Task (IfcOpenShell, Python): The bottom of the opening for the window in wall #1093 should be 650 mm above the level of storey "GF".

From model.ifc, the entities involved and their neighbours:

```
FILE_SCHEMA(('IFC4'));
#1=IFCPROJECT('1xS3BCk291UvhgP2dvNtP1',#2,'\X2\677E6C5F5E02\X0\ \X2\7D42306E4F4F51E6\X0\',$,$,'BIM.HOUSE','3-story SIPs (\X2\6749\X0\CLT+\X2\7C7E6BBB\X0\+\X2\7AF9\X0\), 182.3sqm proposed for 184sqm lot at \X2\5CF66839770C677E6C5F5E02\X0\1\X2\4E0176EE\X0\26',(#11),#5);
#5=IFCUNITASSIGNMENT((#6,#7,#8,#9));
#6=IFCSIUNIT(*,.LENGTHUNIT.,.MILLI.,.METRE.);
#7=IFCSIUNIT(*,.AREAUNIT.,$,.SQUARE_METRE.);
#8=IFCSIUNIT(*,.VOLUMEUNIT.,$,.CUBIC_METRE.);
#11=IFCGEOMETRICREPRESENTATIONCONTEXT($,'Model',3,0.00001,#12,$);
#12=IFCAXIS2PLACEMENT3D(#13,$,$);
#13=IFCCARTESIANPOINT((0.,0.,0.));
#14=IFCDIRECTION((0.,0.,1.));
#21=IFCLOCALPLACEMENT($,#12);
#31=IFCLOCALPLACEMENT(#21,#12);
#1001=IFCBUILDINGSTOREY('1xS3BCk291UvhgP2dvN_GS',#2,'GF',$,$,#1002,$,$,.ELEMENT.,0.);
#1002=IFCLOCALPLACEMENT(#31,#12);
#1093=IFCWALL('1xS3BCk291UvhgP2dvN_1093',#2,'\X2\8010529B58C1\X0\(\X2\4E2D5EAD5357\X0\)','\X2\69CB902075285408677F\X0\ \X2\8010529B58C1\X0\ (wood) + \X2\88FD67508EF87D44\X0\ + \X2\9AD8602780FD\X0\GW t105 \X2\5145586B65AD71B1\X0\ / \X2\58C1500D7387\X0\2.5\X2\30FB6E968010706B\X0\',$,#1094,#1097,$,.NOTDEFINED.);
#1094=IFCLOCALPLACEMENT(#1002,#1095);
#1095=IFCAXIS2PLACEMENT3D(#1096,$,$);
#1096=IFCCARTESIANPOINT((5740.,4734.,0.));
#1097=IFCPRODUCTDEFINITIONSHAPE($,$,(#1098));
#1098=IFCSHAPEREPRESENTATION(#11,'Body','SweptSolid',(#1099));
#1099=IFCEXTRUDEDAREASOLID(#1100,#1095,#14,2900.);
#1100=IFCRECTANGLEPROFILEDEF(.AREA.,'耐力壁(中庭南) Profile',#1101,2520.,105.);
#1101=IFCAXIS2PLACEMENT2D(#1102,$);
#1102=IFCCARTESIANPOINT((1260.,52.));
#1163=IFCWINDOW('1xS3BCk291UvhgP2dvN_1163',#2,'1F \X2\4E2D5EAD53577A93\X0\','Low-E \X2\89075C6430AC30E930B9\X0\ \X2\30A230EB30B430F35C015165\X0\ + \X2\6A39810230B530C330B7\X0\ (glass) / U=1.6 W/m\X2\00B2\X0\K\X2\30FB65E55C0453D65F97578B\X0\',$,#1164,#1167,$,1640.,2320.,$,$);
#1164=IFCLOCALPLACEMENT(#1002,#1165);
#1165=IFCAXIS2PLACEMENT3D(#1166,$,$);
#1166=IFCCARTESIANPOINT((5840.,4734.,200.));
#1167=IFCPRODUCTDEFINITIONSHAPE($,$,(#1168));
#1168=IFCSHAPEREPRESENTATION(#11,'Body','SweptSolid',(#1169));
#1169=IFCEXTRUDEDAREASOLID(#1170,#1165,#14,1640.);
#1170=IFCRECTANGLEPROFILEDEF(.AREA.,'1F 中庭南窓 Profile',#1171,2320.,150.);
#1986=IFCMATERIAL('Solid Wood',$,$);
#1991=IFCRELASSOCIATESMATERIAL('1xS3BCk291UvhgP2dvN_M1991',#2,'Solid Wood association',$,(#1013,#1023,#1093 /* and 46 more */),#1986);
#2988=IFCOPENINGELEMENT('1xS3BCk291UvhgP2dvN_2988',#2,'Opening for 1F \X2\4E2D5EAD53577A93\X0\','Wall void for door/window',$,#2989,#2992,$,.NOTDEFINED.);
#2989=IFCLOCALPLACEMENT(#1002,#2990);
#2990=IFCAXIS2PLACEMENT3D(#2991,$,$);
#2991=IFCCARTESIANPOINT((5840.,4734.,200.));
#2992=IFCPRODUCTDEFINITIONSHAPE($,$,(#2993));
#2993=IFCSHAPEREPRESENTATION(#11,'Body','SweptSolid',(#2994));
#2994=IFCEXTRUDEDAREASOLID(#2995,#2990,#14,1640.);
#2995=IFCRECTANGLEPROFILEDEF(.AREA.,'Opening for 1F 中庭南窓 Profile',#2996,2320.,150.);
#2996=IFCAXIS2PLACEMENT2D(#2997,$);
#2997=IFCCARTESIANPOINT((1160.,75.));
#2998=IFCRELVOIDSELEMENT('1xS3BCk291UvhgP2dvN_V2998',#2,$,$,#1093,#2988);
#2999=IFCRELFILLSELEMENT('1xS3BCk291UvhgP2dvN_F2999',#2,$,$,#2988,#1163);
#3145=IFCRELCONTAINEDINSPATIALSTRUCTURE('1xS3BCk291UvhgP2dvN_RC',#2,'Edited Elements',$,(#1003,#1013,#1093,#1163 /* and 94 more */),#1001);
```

```python
import numpy as np
import ifcopenshell
import ifcopenshell.api.geometry
import ifcopenshell.geom
import ifcopenshell.util.element
import ifcopenshell.util.placement
import ifcopenshell.util.shape
import ifcopenshell.util.unit

model = ifcopenshell.open("model.ifc")
unit_scale = ifcopenshell.util.unit.calculate_unit_scale(model)

window = model.by_id(1163)
opening = window.FillsVoids[0].RelatingOpeningElement
storey = ifcopenshell.util.element.get_container(window, ifc_class="IfcBuildingStorey")
level = ifcopenshell.util.placement.get_local_placement(storey.ObjectPlacement)[2, 3]

# The opening's origin need not be at the sill, so measure its lowest point.
shape = ifcopenshell.geom.create_shape(ifcopenshell.geom.settings(), opening)
bottom = ifcopenshell.util.shape.get_shape_bottom_elevation(shape, shape.geometry) / unit_scale
dz = level + 0.65 / unit_scale - bottom

shift = np.array([0.0, 0.0, dz])
# The window is not placed relative to its opening, so move both.
for product in (opening, window):
    matrix = ifcopenshell.util.placement.get_local_placement(product.ObjectPlacement)
    matrix[:3, 3] += shift
    ifcopenshell.api.geometry.edit_object_placement(model, product=product, matrix=matrix, is_si=False)

print(f"moved by {dz * unit_scale:+.3f} m")

model.write("model_edited.ifc")
```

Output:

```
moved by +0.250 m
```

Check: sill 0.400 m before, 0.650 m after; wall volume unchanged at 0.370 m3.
